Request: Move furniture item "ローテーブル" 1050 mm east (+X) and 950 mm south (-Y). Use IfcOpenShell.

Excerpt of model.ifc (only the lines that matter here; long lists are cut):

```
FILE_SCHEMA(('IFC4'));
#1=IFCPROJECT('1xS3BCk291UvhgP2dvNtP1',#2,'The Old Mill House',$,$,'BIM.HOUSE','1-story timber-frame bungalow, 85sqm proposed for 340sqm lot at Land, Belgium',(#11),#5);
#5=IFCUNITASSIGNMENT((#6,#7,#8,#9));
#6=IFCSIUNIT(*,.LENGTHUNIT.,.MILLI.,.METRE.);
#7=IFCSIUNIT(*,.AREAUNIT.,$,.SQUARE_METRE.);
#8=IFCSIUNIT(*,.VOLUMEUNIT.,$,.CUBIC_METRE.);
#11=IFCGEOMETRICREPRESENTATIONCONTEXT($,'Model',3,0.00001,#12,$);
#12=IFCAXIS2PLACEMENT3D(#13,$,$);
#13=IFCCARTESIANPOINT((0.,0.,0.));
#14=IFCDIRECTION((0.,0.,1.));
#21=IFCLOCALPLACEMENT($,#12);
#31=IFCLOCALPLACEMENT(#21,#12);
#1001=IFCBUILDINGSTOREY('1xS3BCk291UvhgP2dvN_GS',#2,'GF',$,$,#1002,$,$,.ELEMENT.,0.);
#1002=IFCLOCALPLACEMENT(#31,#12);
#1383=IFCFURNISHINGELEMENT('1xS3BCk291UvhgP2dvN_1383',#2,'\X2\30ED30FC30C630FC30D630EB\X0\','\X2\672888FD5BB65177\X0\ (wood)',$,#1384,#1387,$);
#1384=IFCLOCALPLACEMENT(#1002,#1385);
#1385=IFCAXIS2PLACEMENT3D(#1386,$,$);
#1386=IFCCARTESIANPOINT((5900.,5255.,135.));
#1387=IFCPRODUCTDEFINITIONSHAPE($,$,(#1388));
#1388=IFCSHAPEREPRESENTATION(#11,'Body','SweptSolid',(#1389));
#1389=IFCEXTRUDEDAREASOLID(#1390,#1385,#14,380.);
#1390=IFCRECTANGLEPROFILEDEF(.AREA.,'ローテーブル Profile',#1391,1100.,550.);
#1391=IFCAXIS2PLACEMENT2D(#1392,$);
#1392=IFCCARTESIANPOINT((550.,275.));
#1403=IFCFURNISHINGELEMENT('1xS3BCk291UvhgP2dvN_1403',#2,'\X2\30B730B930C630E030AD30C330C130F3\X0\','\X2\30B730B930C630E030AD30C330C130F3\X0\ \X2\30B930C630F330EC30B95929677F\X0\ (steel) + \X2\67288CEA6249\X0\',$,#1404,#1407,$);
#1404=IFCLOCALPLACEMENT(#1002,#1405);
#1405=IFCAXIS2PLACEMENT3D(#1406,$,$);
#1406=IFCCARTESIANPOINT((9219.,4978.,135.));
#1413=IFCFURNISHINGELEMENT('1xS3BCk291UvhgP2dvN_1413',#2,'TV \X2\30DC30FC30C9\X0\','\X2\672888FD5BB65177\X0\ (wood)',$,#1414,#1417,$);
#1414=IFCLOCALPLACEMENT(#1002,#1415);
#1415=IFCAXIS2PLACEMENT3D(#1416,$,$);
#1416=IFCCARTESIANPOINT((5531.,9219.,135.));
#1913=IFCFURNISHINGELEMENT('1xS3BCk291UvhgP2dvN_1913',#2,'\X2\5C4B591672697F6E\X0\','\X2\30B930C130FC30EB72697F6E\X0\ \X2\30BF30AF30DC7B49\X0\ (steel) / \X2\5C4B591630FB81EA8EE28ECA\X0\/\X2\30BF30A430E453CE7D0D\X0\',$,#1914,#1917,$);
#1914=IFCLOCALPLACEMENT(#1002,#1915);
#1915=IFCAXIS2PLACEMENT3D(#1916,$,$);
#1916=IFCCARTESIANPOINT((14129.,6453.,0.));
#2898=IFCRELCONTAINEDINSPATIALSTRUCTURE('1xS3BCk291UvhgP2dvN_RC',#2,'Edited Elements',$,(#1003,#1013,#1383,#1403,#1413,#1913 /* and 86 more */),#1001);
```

```python
import ifcopenshell
import ifcopenshell.api.geometry
import ifcopenshell.util.placement
import ifcopenshell.util.unit

model = ifcopenshell.open("model.ifc")
unit_scale = ifcopenshell.util.unit.calculate_unit_scale(model)

item = model.by_guid("1xS3BCk291UvhgP2dvN_1383")
matrix = ifcopenshell.util.placement.get_local_placement(item.ObjectPlacement)
matrix[0, 3] += 1.05 / unit_scale
matrix[1, 3] -= 0.95 / unit_scale
ifcopenshell.api.geometry.edit_object_placement(model, product=item, matrix=matrix, is_si=False)

print(ifcopenshell.util.placement.get_local_placement(item.ObjectPlacement).round(3) + 0.0)

model.write("model_rev.ifc")
```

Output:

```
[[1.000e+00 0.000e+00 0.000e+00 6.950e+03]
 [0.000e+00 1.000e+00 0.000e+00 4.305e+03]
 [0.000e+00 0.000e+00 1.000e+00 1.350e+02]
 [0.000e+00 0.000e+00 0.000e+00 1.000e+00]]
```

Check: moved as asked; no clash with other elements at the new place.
